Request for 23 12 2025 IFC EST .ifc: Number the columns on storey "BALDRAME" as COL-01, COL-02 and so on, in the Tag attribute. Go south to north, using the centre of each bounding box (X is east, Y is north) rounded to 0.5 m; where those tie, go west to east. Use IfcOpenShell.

First a look at what the model holds.

```python
import ifcopenshell
import ifcopenshell.util.element
import ifcopenshell.util.placement

model = ifcopenshell.open("23 12 2025 IFC EST .ifc")
print(model.schema)
storey = next(s for s in model.by_type("IfcBuildingStorey") if s.Name == "BALDRAME")
columns = [e for e in ifcopenshell.util.element.get_decomposition(storey) if e.is_a("IfcColumn")]
for e in sorted(columns, key=lambda e: e.id()):
    origin = ifcopenshell.util.placement.get_local_placement(e.ObjectPlacement)[:3, 3]
    print(e.id(), e.Tag, e.Name, origin.round(2) + 0.0, sep=" | ")
```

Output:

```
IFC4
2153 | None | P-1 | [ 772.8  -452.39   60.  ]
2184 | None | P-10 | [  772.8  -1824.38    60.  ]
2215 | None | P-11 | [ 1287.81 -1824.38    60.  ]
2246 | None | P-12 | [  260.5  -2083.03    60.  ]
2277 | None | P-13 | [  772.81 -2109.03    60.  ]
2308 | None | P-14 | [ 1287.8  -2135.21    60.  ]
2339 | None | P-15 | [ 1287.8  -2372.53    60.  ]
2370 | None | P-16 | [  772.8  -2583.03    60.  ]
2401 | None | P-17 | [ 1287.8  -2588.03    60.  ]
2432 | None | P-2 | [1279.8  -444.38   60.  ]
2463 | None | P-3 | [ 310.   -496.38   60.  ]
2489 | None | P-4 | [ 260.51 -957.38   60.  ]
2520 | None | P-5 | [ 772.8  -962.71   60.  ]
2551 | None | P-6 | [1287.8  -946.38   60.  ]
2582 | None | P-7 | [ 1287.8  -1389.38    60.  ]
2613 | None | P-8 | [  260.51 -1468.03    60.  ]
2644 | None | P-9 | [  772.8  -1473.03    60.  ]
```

```python
import ifcopenshell
import ifcopenshell.geom
import ifcopenshell.util.element
import ifcopenshell.util.shape

model = ifcopenshell.open("23 12 2025 IFC EST .ifc")
settings = ifcopenshell.geom.settings()
settings.set("use-world-coords", True)


def centre(element):
    shape = ifcopenshell.geom.create_shape(settings, element)
    return ifcopenshell.util.shape.get_bbox_centroid(shape.geometry)


storey = next(s for s in model.by_type("IfcBuildingStorey") if s.Name == "BALDRAME")
columns = [e for e in ifcopenshell.util.element.get_decomposition(storey) if e.is_a("IfcColumn")]

# Insertion points can sit at a corner or the storey origin, so sort by the geometry (in metres).
centres = {e: centre(e) for e in columns}
columns.sort(key=lambda e: (round(centres[e][1] / 0.5), centres[e][0]))

for i, e in enumerate(columns, start=1):
    number = f"COL-{i:02d}"
    e.Tag = number
    print(e.id(), number)

model.write("23 12 2025 IFC EST -out.ifc")
```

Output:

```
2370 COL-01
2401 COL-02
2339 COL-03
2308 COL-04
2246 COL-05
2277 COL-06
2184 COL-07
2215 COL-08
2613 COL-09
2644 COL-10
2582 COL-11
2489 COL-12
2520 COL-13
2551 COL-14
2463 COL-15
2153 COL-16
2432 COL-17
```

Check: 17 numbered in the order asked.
